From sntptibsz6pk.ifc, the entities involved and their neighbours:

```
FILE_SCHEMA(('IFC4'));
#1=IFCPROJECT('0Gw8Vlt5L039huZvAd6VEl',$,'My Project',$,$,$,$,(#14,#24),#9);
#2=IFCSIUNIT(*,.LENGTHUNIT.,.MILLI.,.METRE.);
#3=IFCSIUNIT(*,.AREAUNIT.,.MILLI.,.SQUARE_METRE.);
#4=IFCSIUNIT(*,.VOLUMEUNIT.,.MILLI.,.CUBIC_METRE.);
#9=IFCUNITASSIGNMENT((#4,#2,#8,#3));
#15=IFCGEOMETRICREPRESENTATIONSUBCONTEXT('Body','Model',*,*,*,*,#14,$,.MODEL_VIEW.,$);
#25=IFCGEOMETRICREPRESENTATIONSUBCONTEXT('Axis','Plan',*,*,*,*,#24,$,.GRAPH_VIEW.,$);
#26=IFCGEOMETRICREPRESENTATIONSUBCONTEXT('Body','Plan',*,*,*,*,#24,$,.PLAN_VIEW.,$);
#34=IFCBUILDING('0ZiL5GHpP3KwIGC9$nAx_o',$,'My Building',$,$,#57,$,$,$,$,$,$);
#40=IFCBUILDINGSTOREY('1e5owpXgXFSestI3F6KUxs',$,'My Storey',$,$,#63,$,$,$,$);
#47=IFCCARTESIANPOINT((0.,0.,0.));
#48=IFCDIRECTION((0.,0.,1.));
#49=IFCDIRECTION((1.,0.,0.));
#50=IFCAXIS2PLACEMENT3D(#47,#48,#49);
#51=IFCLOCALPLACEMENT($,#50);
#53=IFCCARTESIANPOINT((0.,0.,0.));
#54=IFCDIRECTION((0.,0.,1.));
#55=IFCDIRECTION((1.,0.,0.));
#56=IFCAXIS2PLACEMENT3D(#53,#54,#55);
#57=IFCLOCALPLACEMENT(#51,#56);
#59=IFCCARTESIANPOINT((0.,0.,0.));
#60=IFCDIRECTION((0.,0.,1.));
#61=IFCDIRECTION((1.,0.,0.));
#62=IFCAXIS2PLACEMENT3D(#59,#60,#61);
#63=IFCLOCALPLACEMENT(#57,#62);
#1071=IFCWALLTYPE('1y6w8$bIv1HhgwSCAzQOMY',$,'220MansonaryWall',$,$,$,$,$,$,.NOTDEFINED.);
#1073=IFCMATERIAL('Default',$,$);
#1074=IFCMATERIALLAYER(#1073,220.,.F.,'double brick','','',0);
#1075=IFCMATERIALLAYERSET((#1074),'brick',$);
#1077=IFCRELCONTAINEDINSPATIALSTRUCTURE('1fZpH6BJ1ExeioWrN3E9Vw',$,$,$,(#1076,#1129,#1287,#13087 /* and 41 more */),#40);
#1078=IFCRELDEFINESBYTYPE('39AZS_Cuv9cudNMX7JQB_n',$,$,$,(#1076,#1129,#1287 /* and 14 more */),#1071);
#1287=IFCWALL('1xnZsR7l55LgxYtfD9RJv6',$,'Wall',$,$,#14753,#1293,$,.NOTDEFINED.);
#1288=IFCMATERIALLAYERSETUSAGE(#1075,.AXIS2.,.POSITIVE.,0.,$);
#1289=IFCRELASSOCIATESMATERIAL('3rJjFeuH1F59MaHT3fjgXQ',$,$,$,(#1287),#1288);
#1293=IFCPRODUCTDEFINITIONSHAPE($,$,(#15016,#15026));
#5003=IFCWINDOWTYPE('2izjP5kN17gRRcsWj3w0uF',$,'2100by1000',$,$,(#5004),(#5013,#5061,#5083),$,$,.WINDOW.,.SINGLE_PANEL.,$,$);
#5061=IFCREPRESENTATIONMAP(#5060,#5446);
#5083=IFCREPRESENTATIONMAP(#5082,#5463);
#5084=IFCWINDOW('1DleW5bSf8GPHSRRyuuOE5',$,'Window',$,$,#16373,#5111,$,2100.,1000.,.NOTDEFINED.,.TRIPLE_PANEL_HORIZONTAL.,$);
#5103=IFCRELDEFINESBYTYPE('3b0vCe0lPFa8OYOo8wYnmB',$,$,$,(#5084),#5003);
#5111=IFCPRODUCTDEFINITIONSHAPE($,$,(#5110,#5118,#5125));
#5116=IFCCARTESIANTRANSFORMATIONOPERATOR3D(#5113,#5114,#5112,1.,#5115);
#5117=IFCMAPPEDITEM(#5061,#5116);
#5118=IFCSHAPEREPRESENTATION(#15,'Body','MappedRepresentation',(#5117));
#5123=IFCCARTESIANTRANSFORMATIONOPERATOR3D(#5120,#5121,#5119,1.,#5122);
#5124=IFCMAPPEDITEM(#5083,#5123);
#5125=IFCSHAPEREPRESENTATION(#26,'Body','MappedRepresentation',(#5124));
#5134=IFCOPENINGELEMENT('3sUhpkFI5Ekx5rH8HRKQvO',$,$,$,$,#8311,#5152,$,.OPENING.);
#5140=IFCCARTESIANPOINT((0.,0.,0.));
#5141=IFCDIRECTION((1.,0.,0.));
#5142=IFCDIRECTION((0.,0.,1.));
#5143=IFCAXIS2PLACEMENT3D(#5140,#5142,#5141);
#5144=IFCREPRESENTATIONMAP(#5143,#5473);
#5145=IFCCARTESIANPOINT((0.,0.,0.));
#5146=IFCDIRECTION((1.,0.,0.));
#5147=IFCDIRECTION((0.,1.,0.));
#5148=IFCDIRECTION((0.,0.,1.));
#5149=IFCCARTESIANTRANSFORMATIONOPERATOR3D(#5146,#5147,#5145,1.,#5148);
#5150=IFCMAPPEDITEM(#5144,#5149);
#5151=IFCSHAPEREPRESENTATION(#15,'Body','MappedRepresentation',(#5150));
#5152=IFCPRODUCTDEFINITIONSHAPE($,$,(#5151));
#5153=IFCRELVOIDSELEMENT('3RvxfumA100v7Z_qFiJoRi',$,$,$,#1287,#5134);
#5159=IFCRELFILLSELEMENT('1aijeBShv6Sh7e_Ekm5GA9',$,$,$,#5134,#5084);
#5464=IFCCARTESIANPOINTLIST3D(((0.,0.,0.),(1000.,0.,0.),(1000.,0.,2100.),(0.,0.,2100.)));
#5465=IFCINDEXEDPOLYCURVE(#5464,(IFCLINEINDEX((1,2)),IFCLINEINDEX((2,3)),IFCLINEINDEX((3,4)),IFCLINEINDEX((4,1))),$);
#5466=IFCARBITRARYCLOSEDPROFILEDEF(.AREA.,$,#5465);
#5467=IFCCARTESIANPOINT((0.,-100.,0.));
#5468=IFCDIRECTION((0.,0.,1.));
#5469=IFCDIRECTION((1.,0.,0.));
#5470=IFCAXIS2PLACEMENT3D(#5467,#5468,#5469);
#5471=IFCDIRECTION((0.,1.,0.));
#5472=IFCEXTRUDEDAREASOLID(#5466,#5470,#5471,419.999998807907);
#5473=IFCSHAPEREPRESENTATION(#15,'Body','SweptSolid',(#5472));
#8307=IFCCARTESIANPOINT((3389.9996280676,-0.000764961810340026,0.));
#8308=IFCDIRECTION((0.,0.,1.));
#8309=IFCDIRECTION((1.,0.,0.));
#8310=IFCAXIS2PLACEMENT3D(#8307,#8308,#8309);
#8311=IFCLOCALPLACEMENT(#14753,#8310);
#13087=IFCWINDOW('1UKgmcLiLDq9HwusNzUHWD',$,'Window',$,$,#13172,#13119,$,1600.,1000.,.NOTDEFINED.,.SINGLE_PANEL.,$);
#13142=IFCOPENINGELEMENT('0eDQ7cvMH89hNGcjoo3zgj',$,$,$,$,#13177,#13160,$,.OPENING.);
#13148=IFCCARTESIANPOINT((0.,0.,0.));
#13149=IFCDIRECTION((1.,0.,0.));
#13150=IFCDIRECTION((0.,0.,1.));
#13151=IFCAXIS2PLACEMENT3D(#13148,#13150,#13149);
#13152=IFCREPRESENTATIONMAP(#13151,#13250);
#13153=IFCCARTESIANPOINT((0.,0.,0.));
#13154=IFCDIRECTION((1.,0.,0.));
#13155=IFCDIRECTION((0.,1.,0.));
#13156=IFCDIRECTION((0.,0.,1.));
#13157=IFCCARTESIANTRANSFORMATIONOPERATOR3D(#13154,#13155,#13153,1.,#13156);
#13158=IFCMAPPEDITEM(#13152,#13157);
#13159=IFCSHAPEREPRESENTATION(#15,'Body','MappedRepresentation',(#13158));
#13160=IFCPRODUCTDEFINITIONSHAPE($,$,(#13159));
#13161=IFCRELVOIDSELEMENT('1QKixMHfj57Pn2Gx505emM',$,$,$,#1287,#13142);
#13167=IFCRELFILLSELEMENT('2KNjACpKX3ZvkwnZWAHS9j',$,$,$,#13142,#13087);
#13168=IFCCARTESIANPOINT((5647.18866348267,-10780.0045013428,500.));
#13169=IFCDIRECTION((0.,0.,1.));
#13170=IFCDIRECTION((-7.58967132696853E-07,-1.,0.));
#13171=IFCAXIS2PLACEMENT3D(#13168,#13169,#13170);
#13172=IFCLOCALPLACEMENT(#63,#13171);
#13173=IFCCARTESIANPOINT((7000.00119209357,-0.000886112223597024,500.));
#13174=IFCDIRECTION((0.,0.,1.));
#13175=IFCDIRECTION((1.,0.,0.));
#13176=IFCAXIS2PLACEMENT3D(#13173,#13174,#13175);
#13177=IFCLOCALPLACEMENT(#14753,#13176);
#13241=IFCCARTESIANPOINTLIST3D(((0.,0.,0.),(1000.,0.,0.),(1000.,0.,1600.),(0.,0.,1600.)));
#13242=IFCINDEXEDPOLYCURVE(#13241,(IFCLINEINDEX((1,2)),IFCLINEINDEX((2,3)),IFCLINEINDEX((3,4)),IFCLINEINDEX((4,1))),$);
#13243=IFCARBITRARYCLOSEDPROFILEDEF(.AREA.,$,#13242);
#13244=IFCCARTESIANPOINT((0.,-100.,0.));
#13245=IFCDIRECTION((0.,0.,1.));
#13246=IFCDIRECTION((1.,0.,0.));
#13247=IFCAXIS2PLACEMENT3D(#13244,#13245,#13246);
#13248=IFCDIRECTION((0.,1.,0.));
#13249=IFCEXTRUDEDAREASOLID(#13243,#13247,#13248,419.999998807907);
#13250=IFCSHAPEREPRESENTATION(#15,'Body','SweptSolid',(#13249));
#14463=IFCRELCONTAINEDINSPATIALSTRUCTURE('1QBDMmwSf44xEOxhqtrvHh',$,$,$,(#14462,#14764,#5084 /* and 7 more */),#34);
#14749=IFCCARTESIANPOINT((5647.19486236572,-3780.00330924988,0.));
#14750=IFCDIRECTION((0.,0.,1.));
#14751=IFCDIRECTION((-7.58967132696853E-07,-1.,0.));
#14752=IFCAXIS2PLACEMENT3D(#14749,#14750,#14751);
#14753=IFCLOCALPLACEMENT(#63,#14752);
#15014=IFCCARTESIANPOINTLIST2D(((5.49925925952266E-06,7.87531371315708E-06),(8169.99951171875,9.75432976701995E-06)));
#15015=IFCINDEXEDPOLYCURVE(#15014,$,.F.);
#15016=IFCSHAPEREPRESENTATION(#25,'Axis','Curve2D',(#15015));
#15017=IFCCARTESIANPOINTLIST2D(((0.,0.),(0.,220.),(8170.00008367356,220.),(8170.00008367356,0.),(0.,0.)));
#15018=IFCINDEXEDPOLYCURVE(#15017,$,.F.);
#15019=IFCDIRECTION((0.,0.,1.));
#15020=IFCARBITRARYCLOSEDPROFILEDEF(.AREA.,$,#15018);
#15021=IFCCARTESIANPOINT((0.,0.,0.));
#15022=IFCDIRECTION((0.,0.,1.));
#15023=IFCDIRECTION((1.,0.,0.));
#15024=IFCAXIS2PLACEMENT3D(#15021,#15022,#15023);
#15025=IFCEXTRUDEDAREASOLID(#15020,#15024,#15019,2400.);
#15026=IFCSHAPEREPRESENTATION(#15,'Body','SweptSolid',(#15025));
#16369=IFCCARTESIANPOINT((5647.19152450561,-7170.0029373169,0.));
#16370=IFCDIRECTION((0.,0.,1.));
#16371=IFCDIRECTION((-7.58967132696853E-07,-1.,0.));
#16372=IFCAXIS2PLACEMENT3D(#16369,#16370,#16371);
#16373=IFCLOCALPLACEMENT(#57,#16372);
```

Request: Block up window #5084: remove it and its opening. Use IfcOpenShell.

```python
import ifcopenshell
import ifcopenshell.api.feature
import ifcopenshell.api.root
import ifcopenshell.geom
import ifcopenshell.util.shape

model = ifcopenshell.open("sntptibsz6pk.ifc")
settings = ifcopenshell.geom.settings()


def volume(element):
    """Net volume in cubic metres, openings subtracted."""
    shape = ifcopenshell.geom.create_shape(settings, element)
    return ifcopenshell.util.shape.get_volume(shape.geometry)


window = model.by_guid("1DleW5bSf8GPHSRRyuuOE5")
opening = window.FillsVoids[0].RelatingOpeningElement
wall = opening.VoidsElements[0].RelatingBuildingElement
before = volume(wall)

ifcopenshell.api.root.remove_product(model, product=window)
ifcopenshell.api.feature.remove_feature(model, feature=opening)

after = volume(wall)

print(f"wall volume {before:.3f} -> {after:.3f} m3")

model.write("sntptibsz6pk-out.ifc")
```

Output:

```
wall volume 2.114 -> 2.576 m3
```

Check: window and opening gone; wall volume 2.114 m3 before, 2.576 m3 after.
